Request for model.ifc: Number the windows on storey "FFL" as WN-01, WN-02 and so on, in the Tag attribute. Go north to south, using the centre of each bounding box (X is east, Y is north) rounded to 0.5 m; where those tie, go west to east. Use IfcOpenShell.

First a look at what the model holds.

```python
import ifcopenshell
import ifcopenshell.util.element
import ifcopenshell.util.placement

model = ifcopenshell.open("model.ifc")
print(model.schema)
storey = next(s for s in model.by_type("IfcBuildingStorey") if s.Name == "FFL")
windows = [e for e in ifcopenshell.util.element.get_decomposition(storey) if e.is_a("IfcWindow")]
for e in sorted(windows, key=lambda e: e.id()):
    origin = ifcopenshell.util.placement.get_local_placement(e.ObjectPlacement)[:3, 3]
    print(e.id(), e.Tag, e.Name, origin.round(2) + 0.0, sep=" | ")
```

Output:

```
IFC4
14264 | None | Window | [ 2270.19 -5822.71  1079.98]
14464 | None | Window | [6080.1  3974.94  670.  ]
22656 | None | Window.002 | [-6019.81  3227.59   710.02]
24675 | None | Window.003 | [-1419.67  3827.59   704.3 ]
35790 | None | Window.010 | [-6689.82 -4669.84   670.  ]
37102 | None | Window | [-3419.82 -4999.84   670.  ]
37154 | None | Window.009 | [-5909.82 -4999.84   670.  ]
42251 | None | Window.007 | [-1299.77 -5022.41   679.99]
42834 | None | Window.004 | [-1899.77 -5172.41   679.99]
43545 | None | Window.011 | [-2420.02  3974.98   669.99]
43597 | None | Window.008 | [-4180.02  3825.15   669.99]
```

```python
import ifcopenshell
import ifcopenshell.geom
import ifcopenshell.util.element
import ifcopenshell.util.shape

model = ifcopenshell.open("model.ifc")
settings = ifcopenshell.geom.settings()
settings.set("use-world-coords", True)


def centre(element):
    shape = ifcopenshell.geom.create_shape(settings, element)
    return ifcopenshell.util.shape.get_bbox_centroid(shape.geometry)


storey = next(s for s in model.by_type("IfcBuildingStorey") if s.Name == "FFL")
windows = [e for e in ifcopenshell.util.element.get_decomposition(storey) if e.is_a("IfcWindow")]

# Insertion points can sit at a corner or the storey origin, so sort by the geometry (in metres).
centres = {e: centre(e) for e in windows}
windows.sort(key=lambda e: (-round(centres[e][1] / 0.5), centres[e][0]))

for i, e in enumerate(windows, start=1):
    number = f"WN-{i:02d}"
    e.Tag = number
    print(e.id(), number)

model.write("model_updated.ifc")
```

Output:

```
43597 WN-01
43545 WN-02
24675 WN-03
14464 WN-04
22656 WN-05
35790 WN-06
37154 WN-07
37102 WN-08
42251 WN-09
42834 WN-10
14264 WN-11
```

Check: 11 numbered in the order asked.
